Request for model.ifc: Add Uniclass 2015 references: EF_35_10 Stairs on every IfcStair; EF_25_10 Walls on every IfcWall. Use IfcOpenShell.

First a look at what the model holds.

```python
import ifcopenshell

model = ifcopenshell.open("model.ifc")
print(model.schema)
print("classifications:", [c.Name for c in model.by_type("IfcClassification")])
for ifc_class in ("IfcDoor", "IfcRoof", "IfcStair", "IfcWall", "IfcWindow"):
    print(ifc_class, len(model.by_type(ifc_class)))
```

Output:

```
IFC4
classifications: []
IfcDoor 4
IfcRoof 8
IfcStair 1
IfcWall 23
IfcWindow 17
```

```python
import ifcopenshell
import ifcopenshell.api.classification

model = ifcopenshell.open("model.ifc")

system = ifcopenshell.api.classification.add_classification(model, classification="Uniclass 2015")

codes = {
    "IfcStair": ("EF_35_10", "Stairs"),
    "IfcWall": ("EF_25_10", "Walls"),
}
for ifc_class, (code, name) in codes.items():
    products = model.by_type(ifc_class)
    ifcopenshell.api.classification.add_reference(
        model, products=products, classification=system, identification=code, name=name
    )
    print(code, len(products))

model.write("model_updated.ifc")
```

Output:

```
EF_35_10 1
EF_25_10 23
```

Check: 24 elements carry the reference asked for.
